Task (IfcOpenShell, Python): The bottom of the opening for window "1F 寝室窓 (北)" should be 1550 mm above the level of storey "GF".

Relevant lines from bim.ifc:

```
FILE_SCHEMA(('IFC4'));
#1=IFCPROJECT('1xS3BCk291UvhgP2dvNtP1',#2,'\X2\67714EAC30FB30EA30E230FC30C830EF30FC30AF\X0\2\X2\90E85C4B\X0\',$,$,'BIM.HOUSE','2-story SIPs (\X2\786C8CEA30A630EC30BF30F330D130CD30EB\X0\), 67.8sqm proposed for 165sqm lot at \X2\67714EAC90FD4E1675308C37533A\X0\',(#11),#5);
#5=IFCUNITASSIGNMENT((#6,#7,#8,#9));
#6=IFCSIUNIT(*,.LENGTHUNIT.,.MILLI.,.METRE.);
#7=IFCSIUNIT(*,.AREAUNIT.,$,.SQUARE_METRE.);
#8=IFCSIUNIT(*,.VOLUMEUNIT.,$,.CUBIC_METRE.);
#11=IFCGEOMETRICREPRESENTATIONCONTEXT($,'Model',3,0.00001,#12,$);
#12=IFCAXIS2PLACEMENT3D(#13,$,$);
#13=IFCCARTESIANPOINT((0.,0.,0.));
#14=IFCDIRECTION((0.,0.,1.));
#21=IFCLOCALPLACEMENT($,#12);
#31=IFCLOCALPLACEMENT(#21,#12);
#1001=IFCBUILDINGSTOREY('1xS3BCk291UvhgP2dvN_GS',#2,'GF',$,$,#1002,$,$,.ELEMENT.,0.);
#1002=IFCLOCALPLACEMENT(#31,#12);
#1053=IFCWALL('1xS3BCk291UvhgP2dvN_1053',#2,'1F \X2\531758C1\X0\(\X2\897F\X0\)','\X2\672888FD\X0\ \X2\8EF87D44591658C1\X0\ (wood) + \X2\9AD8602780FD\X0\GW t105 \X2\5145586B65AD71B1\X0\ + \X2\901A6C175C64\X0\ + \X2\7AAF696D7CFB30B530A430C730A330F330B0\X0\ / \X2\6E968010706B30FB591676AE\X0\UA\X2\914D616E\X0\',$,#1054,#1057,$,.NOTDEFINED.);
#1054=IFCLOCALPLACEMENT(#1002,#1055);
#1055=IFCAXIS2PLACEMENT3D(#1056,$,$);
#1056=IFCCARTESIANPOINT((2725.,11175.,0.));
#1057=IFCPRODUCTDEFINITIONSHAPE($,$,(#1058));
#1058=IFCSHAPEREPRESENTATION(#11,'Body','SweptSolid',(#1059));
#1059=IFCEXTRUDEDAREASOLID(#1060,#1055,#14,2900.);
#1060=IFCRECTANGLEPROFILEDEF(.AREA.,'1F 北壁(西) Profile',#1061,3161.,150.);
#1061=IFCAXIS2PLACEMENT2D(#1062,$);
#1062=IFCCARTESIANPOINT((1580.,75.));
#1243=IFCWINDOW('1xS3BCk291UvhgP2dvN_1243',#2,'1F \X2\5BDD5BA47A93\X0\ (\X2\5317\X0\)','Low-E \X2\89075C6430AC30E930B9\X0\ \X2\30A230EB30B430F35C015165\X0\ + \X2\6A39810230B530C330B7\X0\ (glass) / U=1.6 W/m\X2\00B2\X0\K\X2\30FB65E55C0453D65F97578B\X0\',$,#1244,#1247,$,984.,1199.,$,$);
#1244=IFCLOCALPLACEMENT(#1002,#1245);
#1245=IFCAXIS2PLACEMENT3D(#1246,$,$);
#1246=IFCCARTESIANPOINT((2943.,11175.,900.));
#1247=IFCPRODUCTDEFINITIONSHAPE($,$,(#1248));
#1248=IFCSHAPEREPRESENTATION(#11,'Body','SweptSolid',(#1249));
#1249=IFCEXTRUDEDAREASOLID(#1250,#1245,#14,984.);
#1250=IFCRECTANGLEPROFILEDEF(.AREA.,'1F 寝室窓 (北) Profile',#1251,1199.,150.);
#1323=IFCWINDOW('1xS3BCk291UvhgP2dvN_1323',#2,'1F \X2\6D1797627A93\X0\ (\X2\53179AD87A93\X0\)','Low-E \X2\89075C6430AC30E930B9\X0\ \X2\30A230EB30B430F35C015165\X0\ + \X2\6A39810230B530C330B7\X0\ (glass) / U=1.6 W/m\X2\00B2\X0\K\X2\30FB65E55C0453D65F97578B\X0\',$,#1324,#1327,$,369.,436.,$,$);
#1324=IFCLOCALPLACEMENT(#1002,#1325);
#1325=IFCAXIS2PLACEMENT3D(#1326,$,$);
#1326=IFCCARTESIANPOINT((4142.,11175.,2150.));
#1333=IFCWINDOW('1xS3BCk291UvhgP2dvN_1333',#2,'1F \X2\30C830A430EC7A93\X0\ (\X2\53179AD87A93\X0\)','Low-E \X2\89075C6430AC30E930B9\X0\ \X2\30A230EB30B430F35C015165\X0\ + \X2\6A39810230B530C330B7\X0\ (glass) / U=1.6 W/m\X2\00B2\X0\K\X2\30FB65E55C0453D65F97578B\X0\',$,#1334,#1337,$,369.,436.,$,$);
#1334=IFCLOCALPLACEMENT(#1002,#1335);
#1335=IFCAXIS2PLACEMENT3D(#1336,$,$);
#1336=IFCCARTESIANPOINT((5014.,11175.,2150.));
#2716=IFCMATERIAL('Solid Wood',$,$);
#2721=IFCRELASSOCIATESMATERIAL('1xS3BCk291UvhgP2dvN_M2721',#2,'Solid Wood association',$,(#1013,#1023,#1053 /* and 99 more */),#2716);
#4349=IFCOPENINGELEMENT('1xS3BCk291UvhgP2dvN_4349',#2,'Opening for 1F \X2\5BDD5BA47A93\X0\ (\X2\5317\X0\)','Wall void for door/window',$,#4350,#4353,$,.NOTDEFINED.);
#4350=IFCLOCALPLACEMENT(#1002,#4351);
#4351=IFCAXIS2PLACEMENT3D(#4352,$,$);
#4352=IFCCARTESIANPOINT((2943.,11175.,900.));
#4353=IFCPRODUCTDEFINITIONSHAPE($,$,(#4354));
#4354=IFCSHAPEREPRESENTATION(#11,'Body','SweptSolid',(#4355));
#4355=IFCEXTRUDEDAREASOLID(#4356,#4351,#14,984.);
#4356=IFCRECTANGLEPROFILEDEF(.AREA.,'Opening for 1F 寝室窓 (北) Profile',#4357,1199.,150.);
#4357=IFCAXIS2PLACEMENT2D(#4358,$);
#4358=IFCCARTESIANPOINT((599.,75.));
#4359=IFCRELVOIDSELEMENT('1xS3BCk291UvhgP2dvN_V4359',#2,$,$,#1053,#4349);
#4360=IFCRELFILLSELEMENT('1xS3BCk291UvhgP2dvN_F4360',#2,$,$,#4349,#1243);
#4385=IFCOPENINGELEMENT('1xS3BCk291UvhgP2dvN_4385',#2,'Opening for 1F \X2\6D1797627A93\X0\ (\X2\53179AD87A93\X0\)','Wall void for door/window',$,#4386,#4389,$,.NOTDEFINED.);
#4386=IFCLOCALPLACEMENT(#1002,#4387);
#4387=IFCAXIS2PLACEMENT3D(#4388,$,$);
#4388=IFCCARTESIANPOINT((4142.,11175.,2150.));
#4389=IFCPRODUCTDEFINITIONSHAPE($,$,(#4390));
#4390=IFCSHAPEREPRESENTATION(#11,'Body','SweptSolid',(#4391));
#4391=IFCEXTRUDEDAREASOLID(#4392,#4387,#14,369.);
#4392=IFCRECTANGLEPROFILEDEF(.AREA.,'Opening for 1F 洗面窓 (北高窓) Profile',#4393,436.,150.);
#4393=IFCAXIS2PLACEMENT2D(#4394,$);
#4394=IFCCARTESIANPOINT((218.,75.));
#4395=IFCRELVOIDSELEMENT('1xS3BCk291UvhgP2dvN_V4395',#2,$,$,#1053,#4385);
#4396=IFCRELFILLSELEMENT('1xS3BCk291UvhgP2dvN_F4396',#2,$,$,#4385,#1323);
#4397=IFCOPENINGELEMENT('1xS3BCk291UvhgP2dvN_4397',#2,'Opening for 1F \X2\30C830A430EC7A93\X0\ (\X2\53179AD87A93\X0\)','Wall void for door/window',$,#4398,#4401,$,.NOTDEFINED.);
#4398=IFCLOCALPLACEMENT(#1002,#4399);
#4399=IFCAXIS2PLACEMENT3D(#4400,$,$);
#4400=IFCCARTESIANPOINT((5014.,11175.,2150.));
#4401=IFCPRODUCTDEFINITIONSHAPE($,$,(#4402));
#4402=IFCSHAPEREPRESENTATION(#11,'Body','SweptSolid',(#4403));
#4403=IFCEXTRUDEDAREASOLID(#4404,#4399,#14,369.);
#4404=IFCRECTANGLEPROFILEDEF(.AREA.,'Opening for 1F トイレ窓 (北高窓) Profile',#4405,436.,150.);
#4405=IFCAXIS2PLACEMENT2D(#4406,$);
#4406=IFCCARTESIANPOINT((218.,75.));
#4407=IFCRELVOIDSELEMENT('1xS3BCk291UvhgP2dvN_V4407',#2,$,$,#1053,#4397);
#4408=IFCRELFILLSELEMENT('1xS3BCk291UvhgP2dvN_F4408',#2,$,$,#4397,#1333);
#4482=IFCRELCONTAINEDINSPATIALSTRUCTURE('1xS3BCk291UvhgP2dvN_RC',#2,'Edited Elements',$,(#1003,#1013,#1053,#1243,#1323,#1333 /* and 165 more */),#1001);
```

```python
import numpy as np
import ifcopenshell
import ifcopenshell.api.geometry
import ifcopenshell.geom
import ifcopenshell.util.element
import ifcopenshell.util.placement
import ifcopenshell.util.shape
import ifcopenshell.util.unit

model = ifcopenshell.open("bim.ifc")
unit_scale = ifcopenshell.util.unit.calculate_unit_scale(model)

window = model.by_guid("1xS3BCk291UvhgP2dvN_1243")
opening = window.FillsVoids[0].RelatingOpeningElement
storey = ifcopenshell.util.element.get_container(window, ifc_class="IfcBuildingStorey")
level = ifcopenshell.util.placement.get_local_placement(storey.ObjectPlacement)[2, 3]

# The opening's origin need not be at the sill, so measure its lowest point.
shape = ifcopenshell.geom.create_shape(ifcopenshell.geom.settings(), opening)
bottom = ifcopenshell.util.shape.get_shape_bottom_elevation(shape, shape.geometry) / unit_scale
dz = level + 1.55 / unit_scale - bottom

shift = np.array([0.0, 0.0, dz])
# The window is not placed relative to its opening, so move both.
for product in (opening, window):
    matrix = ifcopenshell.util.placement.get_local_placement(product.ObjectPlacement)
    matrix[:3, 3] += shift
    ifcopenshell.api.geometry.edit_object_placement(model, product=product, matrix=matrix, is_si=False)

print(f"moved by {dz * unit_scale:+.3f} m")

model.write("bim_rev.ifc")
```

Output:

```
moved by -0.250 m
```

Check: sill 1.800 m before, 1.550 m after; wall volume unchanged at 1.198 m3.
